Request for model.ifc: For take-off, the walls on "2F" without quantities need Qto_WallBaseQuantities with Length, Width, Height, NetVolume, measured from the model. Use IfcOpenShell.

First a look at what the model holds.

```python
import ifcopenshell
import ifcopenshell.util.element
import ifcopenshell.util.unit

model = ifcopenshell.open("model.ifc")
print(model.schema)
for unit_type in ("LENGTHUNIT", "AREAUNIT", "VOLUMEUNIT"):
    print(unit_type, ifcopenshell.util.unit.calculate_unit_scale(model, unit_type))
storey = next(s for s in model.by_type("IfcBuildingStorey") if s.Name == "2F")
walls = [e for e in ifcopenshell.util.element.get_decomposition(storey) if e.is_a("IfcWall")]
for e in sorted(walls, key=lambda e: e.id()):
    print(e.id(), e.is_a(), e.Name, list(ifcopenshell.util.element.get_psets(e, qtos_only=True)), sep=" | ")
```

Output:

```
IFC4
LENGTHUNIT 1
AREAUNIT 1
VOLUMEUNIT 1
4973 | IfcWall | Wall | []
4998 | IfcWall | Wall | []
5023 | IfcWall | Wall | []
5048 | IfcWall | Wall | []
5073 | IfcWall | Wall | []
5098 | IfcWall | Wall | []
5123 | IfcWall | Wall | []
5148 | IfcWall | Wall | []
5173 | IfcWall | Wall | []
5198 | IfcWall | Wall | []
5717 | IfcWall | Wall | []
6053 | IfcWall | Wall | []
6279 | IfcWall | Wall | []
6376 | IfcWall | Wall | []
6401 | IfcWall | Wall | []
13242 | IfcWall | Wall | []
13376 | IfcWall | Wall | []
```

```python
import ifcopenshell
import ifcopenshell.api.pset
import ifcopenshell.geom
import ifcopenshell.util.element
import ifcopenshell.util.shape
import ifcopenshell.util.unit

model = ifcopenshell.open("model.ifc")
unit_scale = ifcopenshell.util.unit.calculate_unit_scale(model)
volume_scale = ifcopenshell.util.unit.calculate_unit_scale(model, "VOLUMEUNIT")
settings = ifcopenshell.geom.settings()

storey = next(s for s in model.by_type("IfcBuildingStorey") if s.Name == "2F")
walls = [e for e in ifcopenshell.util.element.get_decomposition(storey) if e.is_a("IfcWall")]

for e in sorted(walls, key=lambda e: e.id()):
    if ifcopenshell.util.element.get_psets(e, qtos_only=True, should_inherit=False):
        continue
    # Geometry comes back in metres, in the element's own axes.
    shape = ifcopenshell.geom.create_shape(settings, e)
    values = {
        "Length": ifcopenshell.util.shape.get_x(shape.geometry) / unit_scale,
        "Width": ifcopenshell.util.shape.get_y(shape.geometry) / unit_scale,
        "Height": ifcopenshell.util.shape.get_z(shape.geometry) / unit_scale,
        "NetVolume": ifcopenshell.util.shape.get_volume(shape.geometry) / volume_scale,
    }
    qto = ifcopenshell.api.pset.add_qto(model, product=e, name="Qto_WallBaseQuantities")
    ifcopenshell.api.pset.edit_qto(model, qto=qto, properties=values)
    print(e.id(), {k: round(v, 3) for k, v in values.items()})

model.write("model_v2.ifc")
```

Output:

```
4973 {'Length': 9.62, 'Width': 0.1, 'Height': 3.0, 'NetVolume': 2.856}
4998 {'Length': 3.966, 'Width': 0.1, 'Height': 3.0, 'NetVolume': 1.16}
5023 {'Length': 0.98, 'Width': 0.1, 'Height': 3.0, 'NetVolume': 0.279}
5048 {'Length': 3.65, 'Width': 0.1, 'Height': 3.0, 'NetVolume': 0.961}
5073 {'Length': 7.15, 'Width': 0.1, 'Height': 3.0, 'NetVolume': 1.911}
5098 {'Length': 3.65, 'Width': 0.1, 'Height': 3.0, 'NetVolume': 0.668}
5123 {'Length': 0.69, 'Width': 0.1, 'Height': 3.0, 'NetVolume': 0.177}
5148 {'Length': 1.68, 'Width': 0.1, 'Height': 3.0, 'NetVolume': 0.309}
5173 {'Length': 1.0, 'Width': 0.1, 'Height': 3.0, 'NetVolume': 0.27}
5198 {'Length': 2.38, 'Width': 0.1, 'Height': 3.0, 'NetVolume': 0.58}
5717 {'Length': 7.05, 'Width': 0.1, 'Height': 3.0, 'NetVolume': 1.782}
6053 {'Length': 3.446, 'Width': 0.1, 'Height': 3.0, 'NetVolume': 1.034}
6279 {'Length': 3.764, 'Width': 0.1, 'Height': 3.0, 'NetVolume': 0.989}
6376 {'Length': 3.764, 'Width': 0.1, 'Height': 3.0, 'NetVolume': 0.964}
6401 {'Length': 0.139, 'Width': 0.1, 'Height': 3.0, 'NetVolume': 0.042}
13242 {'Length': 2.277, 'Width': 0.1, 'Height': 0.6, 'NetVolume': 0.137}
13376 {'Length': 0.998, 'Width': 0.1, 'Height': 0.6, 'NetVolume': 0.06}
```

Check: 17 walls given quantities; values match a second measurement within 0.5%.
